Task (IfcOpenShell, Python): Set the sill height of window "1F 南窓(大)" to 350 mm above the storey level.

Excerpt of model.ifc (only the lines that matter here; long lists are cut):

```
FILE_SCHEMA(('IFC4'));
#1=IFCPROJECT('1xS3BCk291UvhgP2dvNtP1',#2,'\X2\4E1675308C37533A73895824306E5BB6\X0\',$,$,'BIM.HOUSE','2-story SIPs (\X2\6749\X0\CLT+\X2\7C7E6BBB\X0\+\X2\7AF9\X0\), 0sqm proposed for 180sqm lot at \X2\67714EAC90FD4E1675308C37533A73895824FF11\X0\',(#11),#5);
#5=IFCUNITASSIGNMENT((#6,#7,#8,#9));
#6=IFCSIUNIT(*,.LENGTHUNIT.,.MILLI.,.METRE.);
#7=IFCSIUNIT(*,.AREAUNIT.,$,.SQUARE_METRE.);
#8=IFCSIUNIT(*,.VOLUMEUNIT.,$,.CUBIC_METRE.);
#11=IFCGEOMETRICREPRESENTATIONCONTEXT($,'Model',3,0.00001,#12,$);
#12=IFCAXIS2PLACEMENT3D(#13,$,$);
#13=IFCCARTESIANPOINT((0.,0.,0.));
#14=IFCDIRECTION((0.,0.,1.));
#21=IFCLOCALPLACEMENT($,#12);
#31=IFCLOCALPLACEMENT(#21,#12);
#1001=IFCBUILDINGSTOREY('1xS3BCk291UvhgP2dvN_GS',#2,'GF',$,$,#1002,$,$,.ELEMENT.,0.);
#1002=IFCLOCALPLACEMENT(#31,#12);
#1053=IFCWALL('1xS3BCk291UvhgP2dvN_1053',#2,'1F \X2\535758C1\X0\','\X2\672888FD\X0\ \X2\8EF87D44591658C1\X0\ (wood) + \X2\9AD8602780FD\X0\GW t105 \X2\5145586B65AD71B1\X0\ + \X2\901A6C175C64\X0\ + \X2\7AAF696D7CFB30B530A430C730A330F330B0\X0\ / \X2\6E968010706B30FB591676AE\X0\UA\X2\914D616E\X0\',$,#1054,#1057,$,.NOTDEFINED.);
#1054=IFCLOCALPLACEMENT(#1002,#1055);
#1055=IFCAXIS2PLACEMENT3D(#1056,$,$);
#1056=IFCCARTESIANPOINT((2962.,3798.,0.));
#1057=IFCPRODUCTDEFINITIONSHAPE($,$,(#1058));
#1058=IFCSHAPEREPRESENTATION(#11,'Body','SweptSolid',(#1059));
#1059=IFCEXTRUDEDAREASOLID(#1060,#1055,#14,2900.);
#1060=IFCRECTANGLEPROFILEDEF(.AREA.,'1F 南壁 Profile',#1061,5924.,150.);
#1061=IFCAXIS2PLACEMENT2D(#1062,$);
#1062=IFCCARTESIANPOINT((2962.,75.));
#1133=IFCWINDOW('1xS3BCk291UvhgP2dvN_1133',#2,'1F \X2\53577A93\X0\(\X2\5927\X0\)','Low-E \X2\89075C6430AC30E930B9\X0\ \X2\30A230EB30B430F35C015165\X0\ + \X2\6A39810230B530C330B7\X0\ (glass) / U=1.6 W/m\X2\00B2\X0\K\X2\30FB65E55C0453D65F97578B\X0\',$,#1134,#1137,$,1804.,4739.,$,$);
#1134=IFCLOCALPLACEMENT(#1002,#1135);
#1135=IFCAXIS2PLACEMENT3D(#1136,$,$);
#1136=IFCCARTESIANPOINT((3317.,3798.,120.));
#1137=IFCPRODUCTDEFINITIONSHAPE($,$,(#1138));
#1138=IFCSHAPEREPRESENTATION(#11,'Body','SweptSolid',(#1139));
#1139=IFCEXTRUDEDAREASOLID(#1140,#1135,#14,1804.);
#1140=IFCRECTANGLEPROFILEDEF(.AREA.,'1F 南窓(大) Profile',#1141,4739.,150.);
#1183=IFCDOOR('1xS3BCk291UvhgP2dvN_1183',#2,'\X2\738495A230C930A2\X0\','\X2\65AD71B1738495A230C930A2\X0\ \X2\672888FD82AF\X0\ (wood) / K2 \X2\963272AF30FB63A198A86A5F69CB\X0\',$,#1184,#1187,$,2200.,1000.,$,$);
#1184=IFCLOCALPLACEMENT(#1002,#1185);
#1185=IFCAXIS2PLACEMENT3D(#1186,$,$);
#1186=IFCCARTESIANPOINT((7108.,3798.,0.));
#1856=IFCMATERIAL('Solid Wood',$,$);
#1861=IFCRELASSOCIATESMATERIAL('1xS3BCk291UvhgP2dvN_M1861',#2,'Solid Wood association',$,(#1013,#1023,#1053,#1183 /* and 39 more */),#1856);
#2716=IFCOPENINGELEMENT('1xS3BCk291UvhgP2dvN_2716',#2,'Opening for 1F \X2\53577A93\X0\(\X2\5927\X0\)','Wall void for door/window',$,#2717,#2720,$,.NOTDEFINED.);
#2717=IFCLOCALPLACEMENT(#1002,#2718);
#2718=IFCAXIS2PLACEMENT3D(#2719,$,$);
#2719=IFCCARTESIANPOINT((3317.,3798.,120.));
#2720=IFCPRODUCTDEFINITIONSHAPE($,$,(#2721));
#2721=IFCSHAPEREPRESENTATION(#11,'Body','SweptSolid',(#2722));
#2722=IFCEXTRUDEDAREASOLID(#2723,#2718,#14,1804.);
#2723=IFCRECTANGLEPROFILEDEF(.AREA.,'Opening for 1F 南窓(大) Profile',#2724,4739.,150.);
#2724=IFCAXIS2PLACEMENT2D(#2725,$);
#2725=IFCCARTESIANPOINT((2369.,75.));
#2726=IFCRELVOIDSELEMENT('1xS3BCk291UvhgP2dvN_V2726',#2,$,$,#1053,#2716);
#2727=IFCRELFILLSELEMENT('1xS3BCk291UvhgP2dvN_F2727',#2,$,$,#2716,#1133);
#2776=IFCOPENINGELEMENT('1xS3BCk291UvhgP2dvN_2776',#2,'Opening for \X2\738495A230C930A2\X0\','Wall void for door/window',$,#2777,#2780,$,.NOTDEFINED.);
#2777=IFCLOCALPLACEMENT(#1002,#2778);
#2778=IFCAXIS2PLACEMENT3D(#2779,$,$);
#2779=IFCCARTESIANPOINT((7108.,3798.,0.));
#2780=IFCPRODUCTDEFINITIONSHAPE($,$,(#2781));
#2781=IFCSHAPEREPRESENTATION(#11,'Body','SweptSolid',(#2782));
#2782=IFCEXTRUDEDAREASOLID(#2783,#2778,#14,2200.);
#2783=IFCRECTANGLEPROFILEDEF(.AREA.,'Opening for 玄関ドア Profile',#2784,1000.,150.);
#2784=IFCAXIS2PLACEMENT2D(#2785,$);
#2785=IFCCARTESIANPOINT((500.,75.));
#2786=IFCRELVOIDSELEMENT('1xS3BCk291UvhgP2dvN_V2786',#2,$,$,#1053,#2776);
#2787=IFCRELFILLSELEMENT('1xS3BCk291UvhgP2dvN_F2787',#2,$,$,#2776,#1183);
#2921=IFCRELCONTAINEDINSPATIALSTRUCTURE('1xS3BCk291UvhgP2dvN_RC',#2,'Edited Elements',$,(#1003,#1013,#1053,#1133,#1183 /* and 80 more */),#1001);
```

```python
import numpy as np
import ifcopenshell
import ifcopenshell.api.geometry
import ifcopenshell.geom
import ifcopenshell.util.element
import ifcopenshell.util.placement
import ifcopenshell.util.shape
import ifcopenshell.util.unit

model = ifcopenshell.open("model.ifc")
unit_scale = ifcopenshell.util.unit.calculate_unit_scale(model)

window = model.by_guid("1xS3BCk291UvhgP2dvN_1133")
opening = window.FillsVoids[0].RelatingOpeningElement
storey = ifcopenshell.util.element.get_container(window, ifc_class="IfcBuildingStorey")
level = ifcopenshell.util.placement.get_local_placement(storey.ObjectPlacement)[2, 3]

# The opening's origin need not be at the sill, so measure its lowest point.
shape = ifcopenshell.geom.create_shape(ifcopenshell.geom.settings(), opening)
bottom = ifcopenshell.util.shape.get_shape_bottom_elevation(shape, shape.geometry) / unit_scale
dz = level + 0.35 / unit_scale - bottom

shift = np.array([0.0, 0.0, dz])
# The window is not placed relative to its opening, so move both.
for product in (opening, window):
    matrix = ifcopenshell.util.placement.get_local_placement(product.ObjectPlacement)
    matrix[:3, 3] += shift
    ifcopenshell.api.geometry.edit_object_placement(model, product=product, matrix=matrix, is_si=False)

print(f"moved by {dz * unit_scale:+.3f} m")

model.write("model_edited.ifc")
```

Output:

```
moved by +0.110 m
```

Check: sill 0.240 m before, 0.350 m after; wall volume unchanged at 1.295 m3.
